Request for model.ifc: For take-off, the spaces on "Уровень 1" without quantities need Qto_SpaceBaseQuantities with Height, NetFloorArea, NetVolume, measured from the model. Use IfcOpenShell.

First a look at what the model holds.

```python
import ifcopenshell
import ifcopenshell.util.element
import ifcopenshell.util.unit

model = ifcopenshell.open("model.ifc")
print(model.schema)
for unit_type in ("LENGTHUNIT", "AREAUNIT", "VOLUMEUNIT"):
    print(unit_type, ifcopenshell.util.unit.calculate_unit_scale(model, unit_type))
storey = next(s for s in model.by_type("IfcBuildingStorey") if s.Name == "Уровень 1")
spaces = [e for e in ifcopenshell.util.element.get_decomposition(storey) if e.is_a("IfcSpace")]
for e in sorted(spaces, key=lambda e: e.id()):
    print(e.id(), e.is_a(), e.Name, list(ifcopenshell.util.element.get_psets(e, qtos_only=True)), sep=" | ")
```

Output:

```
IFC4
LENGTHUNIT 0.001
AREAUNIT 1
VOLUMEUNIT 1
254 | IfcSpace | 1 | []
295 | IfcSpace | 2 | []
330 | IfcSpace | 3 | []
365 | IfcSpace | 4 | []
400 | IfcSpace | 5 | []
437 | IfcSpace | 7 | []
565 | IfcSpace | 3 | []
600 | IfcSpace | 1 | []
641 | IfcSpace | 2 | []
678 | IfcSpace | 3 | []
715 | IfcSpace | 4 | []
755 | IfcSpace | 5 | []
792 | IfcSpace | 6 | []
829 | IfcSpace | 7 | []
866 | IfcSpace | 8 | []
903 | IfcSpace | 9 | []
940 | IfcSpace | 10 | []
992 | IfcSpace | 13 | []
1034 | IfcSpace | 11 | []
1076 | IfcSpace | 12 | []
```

```python
import ifcopenshell
import ifcopenshell.api.pset
import ifcopenshell.geom
import ifcopenshell.util.element
import ifcopenshell.util.shape
import ifcopenshell.util.unit

model = ifcopenshell.open("model.ifc")
unit_scale = ifcopenshell.util.unit.calculate_unit_scale(model)
area_scale = ifcopenshell.util.unit.calculate_unit_scale(model, "AREAUNIT")
volume_scale = ifcopenshell.util.unit.calculate_unit_scale(model, "VOLUMEUNIT")
settings = ifcopenshell.geom.settings()

storey = next(s for s in model.by_type("IfcBuildingStorey") if s.Name == "Уровень 1")
spaces = [e for e in ifcopenshell.util.element.get_decomposition(storey) if e.is_a("IfcSpace")]

for e in sorted(spaces, key=lambda e: e.id()):
    if ifcopenshell.util.element.get_psets(e, qtos_only=True, should_inherit=False):
        continue
    # Geometry comes back in metres, in the element's own axes.
    shape = ifcopenshell.geom.create_shape(settings, e)
    values = {
        "Height": ifcopenshell.util.shape.get_z(shape.geometry) / unit_scale,
        "NetFloorArea": ifcopenshell.util.shape.get_footprint_area(shape.geometry) / area_scale,
        "NetVolume": ifcopenshell.util.shape.get_volume(shape.geometry) / volume_scale,
    }
    qto = ifcopenshell.api.pset.add_qto(model, product=e, name="Qto_SpaceBaseQuantities")
    ifcopenshell.api.pset.edit_qto(model, qto=qto, properties=values)
    print(e.id(), {k: round(v, 3) for k, v in values.items()})

model.write("model_edited.ifc")
```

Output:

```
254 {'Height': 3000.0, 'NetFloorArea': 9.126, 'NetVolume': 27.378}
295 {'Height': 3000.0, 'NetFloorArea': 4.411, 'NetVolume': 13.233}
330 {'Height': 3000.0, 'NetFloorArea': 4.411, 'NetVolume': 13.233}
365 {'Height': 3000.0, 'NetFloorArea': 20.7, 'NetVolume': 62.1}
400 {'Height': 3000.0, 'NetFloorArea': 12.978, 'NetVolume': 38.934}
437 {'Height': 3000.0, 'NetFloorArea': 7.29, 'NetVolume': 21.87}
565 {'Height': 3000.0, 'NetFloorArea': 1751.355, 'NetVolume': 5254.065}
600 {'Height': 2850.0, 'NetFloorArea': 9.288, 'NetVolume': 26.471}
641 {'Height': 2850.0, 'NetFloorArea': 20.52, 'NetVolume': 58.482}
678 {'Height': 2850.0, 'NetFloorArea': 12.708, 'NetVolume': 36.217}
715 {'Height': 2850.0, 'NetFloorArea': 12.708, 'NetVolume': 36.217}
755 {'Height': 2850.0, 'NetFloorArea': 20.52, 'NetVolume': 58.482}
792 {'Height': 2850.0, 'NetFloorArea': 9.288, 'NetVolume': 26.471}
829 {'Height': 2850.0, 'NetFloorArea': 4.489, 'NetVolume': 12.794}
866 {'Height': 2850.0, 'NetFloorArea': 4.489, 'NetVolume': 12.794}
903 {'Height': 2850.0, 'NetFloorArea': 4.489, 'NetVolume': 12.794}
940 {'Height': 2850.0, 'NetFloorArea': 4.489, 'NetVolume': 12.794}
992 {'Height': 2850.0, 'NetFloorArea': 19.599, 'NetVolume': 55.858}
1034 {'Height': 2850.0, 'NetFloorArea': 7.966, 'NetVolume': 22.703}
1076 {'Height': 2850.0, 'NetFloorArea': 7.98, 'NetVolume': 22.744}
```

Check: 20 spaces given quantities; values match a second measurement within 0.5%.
